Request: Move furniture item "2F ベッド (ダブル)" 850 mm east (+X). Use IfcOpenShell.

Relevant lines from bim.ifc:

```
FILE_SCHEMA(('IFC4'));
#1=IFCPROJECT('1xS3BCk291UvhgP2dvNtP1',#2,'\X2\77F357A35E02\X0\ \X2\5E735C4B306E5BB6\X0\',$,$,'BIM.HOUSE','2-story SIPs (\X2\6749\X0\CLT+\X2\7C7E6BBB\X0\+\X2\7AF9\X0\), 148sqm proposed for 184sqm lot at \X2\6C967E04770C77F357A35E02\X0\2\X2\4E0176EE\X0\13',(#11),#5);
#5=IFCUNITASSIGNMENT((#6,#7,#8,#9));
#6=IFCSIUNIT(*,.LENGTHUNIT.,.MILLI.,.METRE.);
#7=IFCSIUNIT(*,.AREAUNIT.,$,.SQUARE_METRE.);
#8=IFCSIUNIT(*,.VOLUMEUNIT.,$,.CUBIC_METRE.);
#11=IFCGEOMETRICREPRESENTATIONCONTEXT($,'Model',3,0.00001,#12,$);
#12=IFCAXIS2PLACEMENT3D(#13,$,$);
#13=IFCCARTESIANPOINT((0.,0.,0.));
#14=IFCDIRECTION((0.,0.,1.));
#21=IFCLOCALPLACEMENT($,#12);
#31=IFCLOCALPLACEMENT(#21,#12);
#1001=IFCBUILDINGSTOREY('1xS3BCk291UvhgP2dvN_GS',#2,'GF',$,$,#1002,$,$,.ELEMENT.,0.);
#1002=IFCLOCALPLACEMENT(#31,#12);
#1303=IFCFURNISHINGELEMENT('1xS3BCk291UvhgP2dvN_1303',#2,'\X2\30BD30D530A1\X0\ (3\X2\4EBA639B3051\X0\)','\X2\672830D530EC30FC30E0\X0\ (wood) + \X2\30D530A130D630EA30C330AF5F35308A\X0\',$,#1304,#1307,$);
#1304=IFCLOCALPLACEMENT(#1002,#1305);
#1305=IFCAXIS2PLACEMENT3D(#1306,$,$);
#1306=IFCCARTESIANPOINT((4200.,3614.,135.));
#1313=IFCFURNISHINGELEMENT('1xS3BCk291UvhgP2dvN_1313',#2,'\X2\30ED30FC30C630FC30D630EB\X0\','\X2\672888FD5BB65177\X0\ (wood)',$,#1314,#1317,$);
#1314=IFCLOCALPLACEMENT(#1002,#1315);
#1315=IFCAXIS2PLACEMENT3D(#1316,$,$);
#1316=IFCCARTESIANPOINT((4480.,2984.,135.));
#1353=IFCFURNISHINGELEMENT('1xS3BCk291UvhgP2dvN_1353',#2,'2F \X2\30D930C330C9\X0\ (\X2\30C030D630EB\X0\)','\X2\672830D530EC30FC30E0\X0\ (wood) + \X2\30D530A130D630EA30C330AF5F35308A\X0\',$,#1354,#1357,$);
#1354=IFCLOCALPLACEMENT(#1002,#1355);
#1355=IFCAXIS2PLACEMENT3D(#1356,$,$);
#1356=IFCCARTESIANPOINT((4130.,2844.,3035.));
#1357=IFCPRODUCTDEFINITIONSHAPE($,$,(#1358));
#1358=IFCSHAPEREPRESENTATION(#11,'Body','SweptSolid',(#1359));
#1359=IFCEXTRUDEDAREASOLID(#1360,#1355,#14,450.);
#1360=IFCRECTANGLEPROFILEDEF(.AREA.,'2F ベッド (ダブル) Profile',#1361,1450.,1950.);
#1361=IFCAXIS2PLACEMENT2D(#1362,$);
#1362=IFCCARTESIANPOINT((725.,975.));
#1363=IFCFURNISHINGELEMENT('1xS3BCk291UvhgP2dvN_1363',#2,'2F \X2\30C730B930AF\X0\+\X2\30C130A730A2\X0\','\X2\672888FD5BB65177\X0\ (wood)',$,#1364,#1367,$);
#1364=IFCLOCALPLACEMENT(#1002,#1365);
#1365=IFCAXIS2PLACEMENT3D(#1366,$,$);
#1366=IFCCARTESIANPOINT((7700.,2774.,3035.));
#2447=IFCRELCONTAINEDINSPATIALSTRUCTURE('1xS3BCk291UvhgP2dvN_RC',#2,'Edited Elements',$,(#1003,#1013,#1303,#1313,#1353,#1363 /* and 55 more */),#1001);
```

```python
import ifcopenshell
import ifcopenshell.api.geometry
import ifcopenshell.util.placement

model = ifcopenshell.open("bim.ifc")

item = model.by_id(1353)
matrix = ifcopenshell.util.placement.get_local_placement(item.ObjectPlacement)
matrix[0, 3] += 850.0
ifcopenshell.api.geometry.edit_object_placement(model, product=item, matrix=matrix, is_si=False)

print(ifcopenshell.util.placement.get_local_placement(item.ObjectPlacement).round(3) + 0.0)

model.write("bim_rev.ifc")
```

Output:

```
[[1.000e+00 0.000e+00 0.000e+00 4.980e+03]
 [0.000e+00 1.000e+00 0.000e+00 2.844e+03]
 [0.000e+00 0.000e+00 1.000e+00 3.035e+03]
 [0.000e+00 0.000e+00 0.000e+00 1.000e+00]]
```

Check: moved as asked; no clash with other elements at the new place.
